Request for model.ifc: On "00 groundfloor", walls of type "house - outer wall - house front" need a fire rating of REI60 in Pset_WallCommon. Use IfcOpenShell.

First a look at what the model holds.

```python
import ifcopenshell
import ifcopenshell.util.element

model = ifcopenshell.open("model.ifc")
print(model.schema)
storey = next(s for s in model.by_type("IfcBuildingStorey") if s.Name == "00 groundfloor")
walls = [e for e in ifcopenshell.util.element.get_decomposition(storey) if e.is_a("IfcWall")]
seen = {}
for e in walls:
    element_type = ifcopenshell.util.element.get_type(e)
    key = (element_type.Name if element_type != e and element_type else None, ifcopenshell.util.element.get_pset(e, "Pset_WallCommon", "FireRating"))
    seen[key] = seen.get(key, 0) + 1
for (name, value), count in sorted(seen.items(), key=str):
    print(count, "x", name, "|", value)
```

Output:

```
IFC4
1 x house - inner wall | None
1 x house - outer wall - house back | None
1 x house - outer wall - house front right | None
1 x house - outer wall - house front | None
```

```python
import ifcopenshell
import ifcopenshell.api.pset
import ifcopenshell.util.element

model = ifcopenshell.open("model.ifc")

storey = next(s for s in model.by_type("IfcBuildingStorey") if s.Name == "00 groundfloor")
walls = [e for e in ifcopenshell.util.element.get_decomposition(storey) if e.is_a("IfcWall")]

count = 0
for e in walls:
    element_type = ifcopenshell.util.element.get_type(e)
    if element_type in (None, e) or element_type.Name != "house - outer wall - house front":
        continue
    # add_pset returns the element's existing set when there is one.
    pset = ifcopenshell.api.pset.add_pset(model, product=e, name="Pset_WallCommon")
    ifcopenshell.api.pset.edit_pset(model, pset=pset, properties={"FireRating": "REI60"})
    count += 1

print(count, "walls updated")

model.write("model_v2.ifc")
```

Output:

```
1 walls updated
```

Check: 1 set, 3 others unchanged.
